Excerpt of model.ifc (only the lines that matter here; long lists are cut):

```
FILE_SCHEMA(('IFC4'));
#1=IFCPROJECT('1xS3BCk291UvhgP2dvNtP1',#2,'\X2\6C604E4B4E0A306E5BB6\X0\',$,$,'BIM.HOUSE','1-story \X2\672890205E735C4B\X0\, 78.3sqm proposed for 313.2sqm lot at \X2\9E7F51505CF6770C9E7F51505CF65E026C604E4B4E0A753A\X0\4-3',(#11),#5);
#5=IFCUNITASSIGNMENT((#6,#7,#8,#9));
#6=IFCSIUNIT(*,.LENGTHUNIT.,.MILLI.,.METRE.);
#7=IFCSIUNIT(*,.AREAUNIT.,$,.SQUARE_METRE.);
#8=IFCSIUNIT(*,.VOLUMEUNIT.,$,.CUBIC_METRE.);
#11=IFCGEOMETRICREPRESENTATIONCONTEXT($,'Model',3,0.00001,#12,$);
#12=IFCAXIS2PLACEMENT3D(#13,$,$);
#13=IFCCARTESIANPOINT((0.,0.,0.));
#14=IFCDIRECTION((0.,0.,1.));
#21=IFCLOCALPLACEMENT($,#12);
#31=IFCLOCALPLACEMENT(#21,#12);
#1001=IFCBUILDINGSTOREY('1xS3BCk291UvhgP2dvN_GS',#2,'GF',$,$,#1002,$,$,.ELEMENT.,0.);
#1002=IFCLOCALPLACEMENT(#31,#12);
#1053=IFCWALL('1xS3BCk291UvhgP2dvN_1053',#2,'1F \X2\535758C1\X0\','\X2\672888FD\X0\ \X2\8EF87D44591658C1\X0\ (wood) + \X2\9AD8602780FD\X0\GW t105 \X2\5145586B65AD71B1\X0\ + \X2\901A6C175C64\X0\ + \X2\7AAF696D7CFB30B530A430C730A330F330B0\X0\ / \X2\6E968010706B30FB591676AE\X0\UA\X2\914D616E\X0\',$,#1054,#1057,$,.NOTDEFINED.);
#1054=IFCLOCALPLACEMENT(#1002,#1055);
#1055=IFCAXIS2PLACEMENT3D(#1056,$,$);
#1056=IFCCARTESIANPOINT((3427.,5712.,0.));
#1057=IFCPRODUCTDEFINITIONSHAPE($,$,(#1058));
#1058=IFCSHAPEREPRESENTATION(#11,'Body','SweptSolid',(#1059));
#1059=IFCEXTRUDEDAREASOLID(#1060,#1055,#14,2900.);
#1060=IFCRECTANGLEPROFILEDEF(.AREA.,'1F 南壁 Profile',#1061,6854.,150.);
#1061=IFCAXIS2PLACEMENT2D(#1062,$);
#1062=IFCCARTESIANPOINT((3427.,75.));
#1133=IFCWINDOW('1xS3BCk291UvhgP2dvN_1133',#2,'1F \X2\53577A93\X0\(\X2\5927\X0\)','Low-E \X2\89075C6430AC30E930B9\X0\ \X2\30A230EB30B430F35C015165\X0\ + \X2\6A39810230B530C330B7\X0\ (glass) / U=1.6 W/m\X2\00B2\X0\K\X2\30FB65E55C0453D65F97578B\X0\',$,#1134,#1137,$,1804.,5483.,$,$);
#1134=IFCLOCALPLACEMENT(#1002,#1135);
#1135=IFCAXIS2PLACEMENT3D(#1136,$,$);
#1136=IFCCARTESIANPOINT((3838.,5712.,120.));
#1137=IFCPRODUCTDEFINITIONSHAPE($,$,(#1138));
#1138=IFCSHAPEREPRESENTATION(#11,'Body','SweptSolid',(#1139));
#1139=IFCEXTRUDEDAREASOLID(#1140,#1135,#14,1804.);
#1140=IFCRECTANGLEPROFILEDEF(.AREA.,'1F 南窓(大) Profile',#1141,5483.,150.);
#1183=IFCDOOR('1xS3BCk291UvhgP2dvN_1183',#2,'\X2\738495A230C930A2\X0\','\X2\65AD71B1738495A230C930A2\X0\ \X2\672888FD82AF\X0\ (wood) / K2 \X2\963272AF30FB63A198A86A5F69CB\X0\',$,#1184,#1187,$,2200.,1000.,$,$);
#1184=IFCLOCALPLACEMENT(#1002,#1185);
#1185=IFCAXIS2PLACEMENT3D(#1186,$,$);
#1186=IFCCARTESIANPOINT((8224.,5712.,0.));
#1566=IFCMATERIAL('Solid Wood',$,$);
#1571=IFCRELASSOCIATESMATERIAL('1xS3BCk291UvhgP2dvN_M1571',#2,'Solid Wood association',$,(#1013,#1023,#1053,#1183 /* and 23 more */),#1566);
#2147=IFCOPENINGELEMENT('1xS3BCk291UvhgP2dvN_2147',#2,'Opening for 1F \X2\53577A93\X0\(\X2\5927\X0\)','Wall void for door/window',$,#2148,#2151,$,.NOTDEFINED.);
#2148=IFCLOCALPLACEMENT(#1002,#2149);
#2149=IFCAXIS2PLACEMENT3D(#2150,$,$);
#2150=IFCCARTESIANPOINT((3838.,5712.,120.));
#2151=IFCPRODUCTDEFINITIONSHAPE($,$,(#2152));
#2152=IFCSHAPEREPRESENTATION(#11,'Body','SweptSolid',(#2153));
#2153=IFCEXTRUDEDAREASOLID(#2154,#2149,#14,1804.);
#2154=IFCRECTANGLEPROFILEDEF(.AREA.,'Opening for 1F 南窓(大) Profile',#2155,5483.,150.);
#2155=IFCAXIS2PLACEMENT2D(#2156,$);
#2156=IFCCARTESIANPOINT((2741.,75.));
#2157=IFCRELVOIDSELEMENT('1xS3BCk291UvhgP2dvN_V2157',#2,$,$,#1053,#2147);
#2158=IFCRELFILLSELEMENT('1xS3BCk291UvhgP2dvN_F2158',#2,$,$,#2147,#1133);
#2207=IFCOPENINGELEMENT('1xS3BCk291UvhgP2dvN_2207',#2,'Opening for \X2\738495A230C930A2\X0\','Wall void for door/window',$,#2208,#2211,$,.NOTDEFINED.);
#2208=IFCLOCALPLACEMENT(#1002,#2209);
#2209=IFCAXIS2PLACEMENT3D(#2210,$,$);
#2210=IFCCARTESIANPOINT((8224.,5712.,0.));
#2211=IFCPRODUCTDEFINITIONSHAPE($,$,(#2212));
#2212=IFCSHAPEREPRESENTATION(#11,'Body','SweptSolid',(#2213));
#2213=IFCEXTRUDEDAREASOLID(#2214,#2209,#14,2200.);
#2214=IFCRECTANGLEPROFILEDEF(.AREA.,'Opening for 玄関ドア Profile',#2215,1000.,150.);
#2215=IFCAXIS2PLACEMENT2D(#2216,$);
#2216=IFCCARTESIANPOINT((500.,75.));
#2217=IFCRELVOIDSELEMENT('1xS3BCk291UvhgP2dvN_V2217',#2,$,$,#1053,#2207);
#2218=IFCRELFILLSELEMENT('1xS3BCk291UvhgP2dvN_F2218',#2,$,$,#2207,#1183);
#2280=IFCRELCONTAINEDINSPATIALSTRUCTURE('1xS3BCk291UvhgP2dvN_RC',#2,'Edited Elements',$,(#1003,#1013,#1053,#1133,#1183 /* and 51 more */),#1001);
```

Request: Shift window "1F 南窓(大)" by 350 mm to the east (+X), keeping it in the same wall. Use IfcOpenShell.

```python
import ifcopenshell
import ifcopenshell.api.geometry
import ifcopenshell.util.placement

model = ifcopenshell.open("model.ifc")

window = model.by_guid("1xS3BCk291UvhgP2dvN_1133")
opening = window.FillsVoids[0].RelatingOpeningElement
wall = opening.VoidsElements[0].RelatingBuildingElement

wall_matrix = ifcopenshell.util.placement.get_local_placement(wall.ObjectPlacement)
shift = wall_matrix[:3, 0] * 350.0
before = ifcopenshell.util.placement.get_local_placement(window.ObjectPlacement)[:3, 3].copy()

# The window is not placed relative to its opening, so move both.
for product in (opening, window):
    matrix = ifcopenshell.util.placement.get_local_placement(product.ObjectPlacement)
    matrix[:3, 3] += shift
    ifcopenshell.api.geometry.edit_object_placement(model, product=product, matrix=matrix, is_si=False)

after = ifcopenshell.util.placement.get_local_placement(window.ObjectPlacement)[:3, 3]
print("window moved by", (after - before).round(3) + 0.0)

model.write("model_updated.ifc")
```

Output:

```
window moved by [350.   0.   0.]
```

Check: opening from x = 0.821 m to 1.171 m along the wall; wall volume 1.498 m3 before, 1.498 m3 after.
